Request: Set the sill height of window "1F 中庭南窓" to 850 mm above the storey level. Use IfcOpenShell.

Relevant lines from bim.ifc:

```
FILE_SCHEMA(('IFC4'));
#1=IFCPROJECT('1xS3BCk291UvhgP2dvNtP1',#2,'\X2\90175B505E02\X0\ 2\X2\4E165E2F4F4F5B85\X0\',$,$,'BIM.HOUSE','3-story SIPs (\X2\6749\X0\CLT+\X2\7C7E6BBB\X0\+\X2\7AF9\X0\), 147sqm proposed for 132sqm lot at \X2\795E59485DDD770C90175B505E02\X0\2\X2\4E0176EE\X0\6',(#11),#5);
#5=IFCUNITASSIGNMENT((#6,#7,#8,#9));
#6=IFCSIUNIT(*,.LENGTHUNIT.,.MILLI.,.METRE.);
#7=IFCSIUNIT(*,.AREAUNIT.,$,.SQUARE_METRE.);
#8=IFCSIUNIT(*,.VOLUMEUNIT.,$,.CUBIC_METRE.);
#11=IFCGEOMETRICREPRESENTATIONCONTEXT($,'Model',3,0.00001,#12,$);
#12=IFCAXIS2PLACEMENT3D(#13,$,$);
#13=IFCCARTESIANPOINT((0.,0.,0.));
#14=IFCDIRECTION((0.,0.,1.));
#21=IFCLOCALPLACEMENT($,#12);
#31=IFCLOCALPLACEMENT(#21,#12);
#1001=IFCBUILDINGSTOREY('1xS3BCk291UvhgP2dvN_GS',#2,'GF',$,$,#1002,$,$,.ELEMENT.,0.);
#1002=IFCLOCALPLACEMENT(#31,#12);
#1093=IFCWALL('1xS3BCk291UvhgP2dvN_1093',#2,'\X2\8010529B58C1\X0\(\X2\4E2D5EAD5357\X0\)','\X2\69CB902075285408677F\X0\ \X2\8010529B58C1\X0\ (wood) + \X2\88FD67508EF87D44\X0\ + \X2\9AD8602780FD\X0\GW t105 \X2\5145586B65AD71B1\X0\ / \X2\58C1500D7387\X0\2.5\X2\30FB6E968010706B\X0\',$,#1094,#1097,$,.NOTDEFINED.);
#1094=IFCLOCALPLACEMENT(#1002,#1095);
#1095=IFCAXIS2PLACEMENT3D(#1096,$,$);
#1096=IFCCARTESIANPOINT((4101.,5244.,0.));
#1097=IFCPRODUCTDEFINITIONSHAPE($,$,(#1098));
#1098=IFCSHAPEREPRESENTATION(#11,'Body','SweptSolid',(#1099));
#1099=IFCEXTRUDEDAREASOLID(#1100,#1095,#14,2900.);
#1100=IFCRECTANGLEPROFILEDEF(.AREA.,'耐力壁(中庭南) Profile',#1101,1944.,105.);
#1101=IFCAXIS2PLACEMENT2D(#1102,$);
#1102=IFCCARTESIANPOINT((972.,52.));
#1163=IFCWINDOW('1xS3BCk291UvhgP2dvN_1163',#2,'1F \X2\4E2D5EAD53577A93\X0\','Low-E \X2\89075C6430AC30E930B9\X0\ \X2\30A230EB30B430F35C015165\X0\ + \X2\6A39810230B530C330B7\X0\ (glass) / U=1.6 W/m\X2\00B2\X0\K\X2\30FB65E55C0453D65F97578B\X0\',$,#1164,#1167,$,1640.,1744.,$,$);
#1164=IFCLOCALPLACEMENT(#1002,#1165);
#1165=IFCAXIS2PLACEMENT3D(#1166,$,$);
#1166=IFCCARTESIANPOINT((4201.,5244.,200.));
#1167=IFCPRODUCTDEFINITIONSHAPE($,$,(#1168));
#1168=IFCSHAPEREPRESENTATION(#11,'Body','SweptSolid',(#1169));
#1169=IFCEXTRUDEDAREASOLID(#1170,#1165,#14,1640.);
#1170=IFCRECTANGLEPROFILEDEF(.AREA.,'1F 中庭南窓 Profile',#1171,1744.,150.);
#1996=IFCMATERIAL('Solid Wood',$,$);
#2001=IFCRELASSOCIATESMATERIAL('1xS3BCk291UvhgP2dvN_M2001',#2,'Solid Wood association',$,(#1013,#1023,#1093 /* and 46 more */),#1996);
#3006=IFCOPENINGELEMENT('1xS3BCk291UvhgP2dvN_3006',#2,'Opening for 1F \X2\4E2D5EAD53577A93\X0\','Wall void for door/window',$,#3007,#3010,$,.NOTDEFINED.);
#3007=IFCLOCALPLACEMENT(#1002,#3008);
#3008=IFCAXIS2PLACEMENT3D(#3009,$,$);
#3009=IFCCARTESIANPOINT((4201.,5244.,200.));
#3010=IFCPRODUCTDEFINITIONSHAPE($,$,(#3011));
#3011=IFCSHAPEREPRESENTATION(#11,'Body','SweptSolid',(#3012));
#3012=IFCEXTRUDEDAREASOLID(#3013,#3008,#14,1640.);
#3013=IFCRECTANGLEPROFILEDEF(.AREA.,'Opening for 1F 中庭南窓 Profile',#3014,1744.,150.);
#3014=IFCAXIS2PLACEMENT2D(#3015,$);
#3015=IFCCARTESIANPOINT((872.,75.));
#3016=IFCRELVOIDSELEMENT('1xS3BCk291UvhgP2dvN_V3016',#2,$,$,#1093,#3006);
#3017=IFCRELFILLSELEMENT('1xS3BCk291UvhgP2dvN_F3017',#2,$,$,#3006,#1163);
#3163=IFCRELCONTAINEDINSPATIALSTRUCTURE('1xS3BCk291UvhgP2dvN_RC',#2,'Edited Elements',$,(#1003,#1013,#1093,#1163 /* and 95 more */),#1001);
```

```python
import numpy as np
import ifcopenshell
import ifcopenshell.api.geometry
import ifcopenshell.geom
import ifcopenshell.util.element
import ifcopenshell.util.placement
import ifcopenshell.util.shape
import ifcopenshell.util.unit

model = ifcopenshell.open("bim.ifc")
unit_scale = ifcopenshell.util.unit.calculate_unit_scale(model)

window = model.by_guid("1xS3BCk291UvhgP2dvN_1163")
opening = window.FillsVoids[0].RelatingOpeningElement
storey = ifcopenshell.util.element.get_container(window, ifc_class="IfcBuildingStorey")
level = ifcopenshell.util.placement.get_local_placement(storey.ObjectPlacement)[2, 3]

# The opening's origin need not be at the sill, so measure its lowest point.
shape = ifcopenshell.geom.create_shape(ifcopenshell.geom.settings(), opening)
bottom = ifcopenshell.util.shape.get_shape_bottom_elevation(shape, shape.geometry) / unit_scale
dz = level + 850.0 - bottom

shift = np.array([0.0, 0.0, dz])
# The window is not placed relative to its opening, so move both.
for product in (opening, window):
    matrix = ifcopenshell.util.placement.get_local_placement(product.ObjectPlacement)
    matrix[:3, 3] += shift
    ifcopenshell.api.geometry.edit_object_placement(model, product=product, matrix=matrix, is_si=False)

print(f"moved by {dz * unit_scale:+.3f} m")

model.write("bim_rev.ifc")
```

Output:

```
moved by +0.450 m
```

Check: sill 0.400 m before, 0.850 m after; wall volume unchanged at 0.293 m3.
